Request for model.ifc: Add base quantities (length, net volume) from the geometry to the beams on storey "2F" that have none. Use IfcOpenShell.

First a look at what the model holds.

```python
import ifcopenshell
import ifcopenshell.util.element
import ifcopenshell.util.unit

model = ifcopenshell.open("model.ifc")
print(model.schema)
for unit_type in ("LENGTHUNIT", "AREAUNIT", "VOLUMEUNIT"):
    print(unit_type, ifcopenshell.util.unit.calculate_unit_scale(model, unit_type))
storey = next(s for s in model.by_type("IfcBuildingStorey") if s.Name == "2F")
beams = [e for e in ifcopenshell.util.element.get_decomposition(storey) if e.is_a("IfcBeam")]
for e in sorted(beams, key=lambda e: e.id()):
    print(e.id(), e.is_a(), e.Name, list(ifcopenshell.util.element.get_psets(e, qtos_only=True)), sep=" | ")
```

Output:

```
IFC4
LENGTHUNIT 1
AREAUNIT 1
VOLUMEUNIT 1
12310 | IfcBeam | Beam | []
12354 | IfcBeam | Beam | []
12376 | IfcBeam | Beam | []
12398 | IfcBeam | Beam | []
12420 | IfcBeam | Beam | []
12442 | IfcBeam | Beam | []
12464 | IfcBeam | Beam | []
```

```python
import ifcopenshell
import ifcopenshell.api.pset
import ifcopenshell.geom
import ifcopenshell.util.element
import ifcopenshell.util.shape
import ifcopenshell.util.unit

model = ifcopenshell.open("model.ifc")
unit_scale = ifcopenshell.util.unit.calculate_unit_scale(model)
volume_scale = ifcopenshell.util.unit.calculate_unit_scale(model, "VOLUMEUNIT")
settings = ifcopenshell.geom.settings()

storey = next(s for s in model.by_type("IfcBuildingStorey") if s.Name == "2F")
beams = [e for e in ifcopenshell.util.element.get_decomposition(storey) if e.is_a("IfcBeam")]

for e in sorted(beams, key=lambda e: e.id()):
    if ifcopenshell.util.element.get_psets(e, qtos_only=True, should_inherit=False):
        continue
    # Geometry comes back in metres, in the element's own axes.
    shape = ifcopenshell.geom.create_shape(settings, e)
    values = {
        "Length": ifcopenshell.util.shape.get_max_xyz(shape.geometry) / unit_scale,
        "NetVolume": ifcopenshell.util.shape.get_volume(shape.geometry) / volume_scale,
    }
    qto = ifcopenshell.api.pset.add_qto(model, product=e, name="Qto_BeamBaseQuantities")
    ifcopenshell.api.pset.edit_qto(model, qto=qto, properties=values)
    print(e.id(), {k: round(v, 3) for k, v in values.items()})

model.write("model_v2.ifc")
```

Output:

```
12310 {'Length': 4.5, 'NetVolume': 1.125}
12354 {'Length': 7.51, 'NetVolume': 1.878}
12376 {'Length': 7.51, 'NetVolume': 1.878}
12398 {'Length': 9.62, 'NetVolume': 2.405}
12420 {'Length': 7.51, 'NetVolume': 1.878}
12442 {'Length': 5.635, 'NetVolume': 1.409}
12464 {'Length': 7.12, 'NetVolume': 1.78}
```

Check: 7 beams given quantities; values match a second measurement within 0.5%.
